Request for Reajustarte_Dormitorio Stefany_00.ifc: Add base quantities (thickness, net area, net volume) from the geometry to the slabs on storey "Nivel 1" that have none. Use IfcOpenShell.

First a look at what the model holds.

```python
import ifcopenshell
import ifcopenshell.util.element
import ifcopenshell.util.unit

model = ifcopenshell.open("Reajustarte_Dormitorio Stefany_00.ifc")
print(model.schema)
for unit_type in ("LENGTHUNIT", "AREAUNIT", "VOLUMEUNIT"):
    print(unit_type, ifcopenshell.util.unit.calculate_unit_scale(model, unit_type))
storey = next(s for s in model.by_type("IfcBuildingStorey") if s.Name == "Nivel 1")
slabs = [e for e in ifcopenshell.util.element.get_decomposition(storey) if e.is_a("IfcSlab")]
for e in sorted(slabs, key=lambda e: e.id()):
    print(e.id(), e.is_a(), e.Name, list(ifcopenshell.util.element.get_psets(e, qtos_only=True)), sep=" | ")
```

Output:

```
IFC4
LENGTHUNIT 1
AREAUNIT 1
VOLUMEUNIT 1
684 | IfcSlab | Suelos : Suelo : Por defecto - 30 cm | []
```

```python
import ifcopenshell
import ifcopenshell.api.pset
import ifcopenshell.geom
import ifcopenshell.util.element
import ifcopenshell.util.shape
import ifcopenshell.util.unit

model = ifcopenshell.open("Reajustarte_Dormitorio Stefany_00.ifc")
unit_scale = ifcopenshell.util.unit.calculate_unit_scale(model)
area_scale = ifcopenshell.util.unit.calculate_unit_scale(model, "AREAUNIT")
volume_scale = ifcopenshell.util.unit.calculate_unit_scale(model, "VOLUMEUNIT")
settings = ifcopenshell.geom.settings()

storey = next(s for s in model.by_type("IfcBuildingStorey") if s.Name == "Nivel 1")
slabs = [e for e in ifcopenshell.util.element.get_decomposition(storey) if e.is_a("IfcSlab")]

for e in sorted(slabs, key=lambda e: e.id()):
    if ifcopenshell.util.element.get_psets(e, qtos_only=True, should_inherit=False):
        continue
    # Geometry comes back in metres, in the element's own axes.
    shape = ifcopenshell.geom.create_shape(settings, e)
    values = {
        "Width": ifcopenshell.util.shape.get_z(shape.geometry) / unit_scale,
        "NetArea": ifcopenshell.util.shape.get_footprint_area(shape.geometry) / area_scale,
        "NetVolume": ifcopenshell.util.shape.get_volume(shape.geometry) / volume_scale,
    }
    qto = ifcopenshell.api.pset.add_qto(model, product=e, name="Qto_SlabBaseQuantities")
    ifcopenshell.api.pset.edit_qto(model, qto=qto, properties=values)
    print(e.id(), {k: round(v, 3) for k, v in values.items()})

model.write("Reajustarte_Dormitorio Stefany_00-out.ifc")
```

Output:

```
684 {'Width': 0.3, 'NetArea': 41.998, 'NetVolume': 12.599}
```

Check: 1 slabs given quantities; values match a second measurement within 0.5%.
